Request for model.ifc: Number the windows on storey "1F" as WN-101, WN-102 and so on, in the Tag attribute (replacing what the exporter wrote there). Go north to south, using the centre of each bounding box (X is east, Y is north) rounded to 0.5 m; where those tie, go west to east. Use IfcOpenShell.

First a look at what the model holds.

```python
import ifcopenshell
import ifcopenshell.util.element
import ifcopenshell.util.placement

model = ifcopenshell.open("model.ifc")
print(model.schema)
storey = next(s for s in model.by_type("IfcBuildingStorey") if s.Name == "1F")
windows = [e for e in ifcopenshell.util.element.get_decomposition(storey) if e.is_a("IfcWindow")]
for e in sorted(windows, key=lambda e: e.id()):
    origin = ifcopenshell.util.placement.get_local_placement(e.ObjectPlacement)[:3, 3]
    print(e.id(), e.Tag, e.Name, origin.round(2) + 0.0, sep=" | ")
```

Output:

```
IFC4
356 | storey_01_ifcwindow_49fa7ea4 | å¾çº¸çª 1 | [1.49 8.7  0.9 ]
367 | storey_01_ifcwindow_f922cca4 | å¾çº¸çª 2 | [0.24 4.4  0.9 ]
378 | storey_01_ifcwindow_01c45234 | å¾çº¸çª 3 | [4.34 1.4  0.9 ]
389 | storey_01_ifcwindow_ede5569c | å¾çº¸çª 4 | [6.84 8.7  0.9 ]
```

```python
import ifcopenshell
import ifcopenshell.geom
import ifcopenshell.util.element
import ifcopenshell.util.shape

model = ifcopenshell.open("model.ifc")
settings = ifcopenshell.geom.settings()
settings.set("use-world-coords", True)


def centre(element):
    shape = ifcopenshell.geom.create_shape(settings, element)
    return ifcopenshell.util.shape.get_bbox_centroid(shape.geometry)


storey = next(s for s in model.by_type("IfcBuildingStorey") if s.Name == "1F")
windows = [e for e in ifcopenshell.util.element.get_decomposition(storey) if e.is_a("IfcWindow")]

# Insertion points can sit at a corner or the storey origin, so sort by the geometry (in metres).
centres = {e: centre(e) for e in windows}
windows.sort(key=lambda e: (-round(centres[e][1] / 0.5), centres[e][0]))

for i, e in enumerate(windows, start=1):
    number = f"WN-1{i:02d}"
    e.Tag = number
    print(e.id(), number)

model.write("model_rev.ifc")
```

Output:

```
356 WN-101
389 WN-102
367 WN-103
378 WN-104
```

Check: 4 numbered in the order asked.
